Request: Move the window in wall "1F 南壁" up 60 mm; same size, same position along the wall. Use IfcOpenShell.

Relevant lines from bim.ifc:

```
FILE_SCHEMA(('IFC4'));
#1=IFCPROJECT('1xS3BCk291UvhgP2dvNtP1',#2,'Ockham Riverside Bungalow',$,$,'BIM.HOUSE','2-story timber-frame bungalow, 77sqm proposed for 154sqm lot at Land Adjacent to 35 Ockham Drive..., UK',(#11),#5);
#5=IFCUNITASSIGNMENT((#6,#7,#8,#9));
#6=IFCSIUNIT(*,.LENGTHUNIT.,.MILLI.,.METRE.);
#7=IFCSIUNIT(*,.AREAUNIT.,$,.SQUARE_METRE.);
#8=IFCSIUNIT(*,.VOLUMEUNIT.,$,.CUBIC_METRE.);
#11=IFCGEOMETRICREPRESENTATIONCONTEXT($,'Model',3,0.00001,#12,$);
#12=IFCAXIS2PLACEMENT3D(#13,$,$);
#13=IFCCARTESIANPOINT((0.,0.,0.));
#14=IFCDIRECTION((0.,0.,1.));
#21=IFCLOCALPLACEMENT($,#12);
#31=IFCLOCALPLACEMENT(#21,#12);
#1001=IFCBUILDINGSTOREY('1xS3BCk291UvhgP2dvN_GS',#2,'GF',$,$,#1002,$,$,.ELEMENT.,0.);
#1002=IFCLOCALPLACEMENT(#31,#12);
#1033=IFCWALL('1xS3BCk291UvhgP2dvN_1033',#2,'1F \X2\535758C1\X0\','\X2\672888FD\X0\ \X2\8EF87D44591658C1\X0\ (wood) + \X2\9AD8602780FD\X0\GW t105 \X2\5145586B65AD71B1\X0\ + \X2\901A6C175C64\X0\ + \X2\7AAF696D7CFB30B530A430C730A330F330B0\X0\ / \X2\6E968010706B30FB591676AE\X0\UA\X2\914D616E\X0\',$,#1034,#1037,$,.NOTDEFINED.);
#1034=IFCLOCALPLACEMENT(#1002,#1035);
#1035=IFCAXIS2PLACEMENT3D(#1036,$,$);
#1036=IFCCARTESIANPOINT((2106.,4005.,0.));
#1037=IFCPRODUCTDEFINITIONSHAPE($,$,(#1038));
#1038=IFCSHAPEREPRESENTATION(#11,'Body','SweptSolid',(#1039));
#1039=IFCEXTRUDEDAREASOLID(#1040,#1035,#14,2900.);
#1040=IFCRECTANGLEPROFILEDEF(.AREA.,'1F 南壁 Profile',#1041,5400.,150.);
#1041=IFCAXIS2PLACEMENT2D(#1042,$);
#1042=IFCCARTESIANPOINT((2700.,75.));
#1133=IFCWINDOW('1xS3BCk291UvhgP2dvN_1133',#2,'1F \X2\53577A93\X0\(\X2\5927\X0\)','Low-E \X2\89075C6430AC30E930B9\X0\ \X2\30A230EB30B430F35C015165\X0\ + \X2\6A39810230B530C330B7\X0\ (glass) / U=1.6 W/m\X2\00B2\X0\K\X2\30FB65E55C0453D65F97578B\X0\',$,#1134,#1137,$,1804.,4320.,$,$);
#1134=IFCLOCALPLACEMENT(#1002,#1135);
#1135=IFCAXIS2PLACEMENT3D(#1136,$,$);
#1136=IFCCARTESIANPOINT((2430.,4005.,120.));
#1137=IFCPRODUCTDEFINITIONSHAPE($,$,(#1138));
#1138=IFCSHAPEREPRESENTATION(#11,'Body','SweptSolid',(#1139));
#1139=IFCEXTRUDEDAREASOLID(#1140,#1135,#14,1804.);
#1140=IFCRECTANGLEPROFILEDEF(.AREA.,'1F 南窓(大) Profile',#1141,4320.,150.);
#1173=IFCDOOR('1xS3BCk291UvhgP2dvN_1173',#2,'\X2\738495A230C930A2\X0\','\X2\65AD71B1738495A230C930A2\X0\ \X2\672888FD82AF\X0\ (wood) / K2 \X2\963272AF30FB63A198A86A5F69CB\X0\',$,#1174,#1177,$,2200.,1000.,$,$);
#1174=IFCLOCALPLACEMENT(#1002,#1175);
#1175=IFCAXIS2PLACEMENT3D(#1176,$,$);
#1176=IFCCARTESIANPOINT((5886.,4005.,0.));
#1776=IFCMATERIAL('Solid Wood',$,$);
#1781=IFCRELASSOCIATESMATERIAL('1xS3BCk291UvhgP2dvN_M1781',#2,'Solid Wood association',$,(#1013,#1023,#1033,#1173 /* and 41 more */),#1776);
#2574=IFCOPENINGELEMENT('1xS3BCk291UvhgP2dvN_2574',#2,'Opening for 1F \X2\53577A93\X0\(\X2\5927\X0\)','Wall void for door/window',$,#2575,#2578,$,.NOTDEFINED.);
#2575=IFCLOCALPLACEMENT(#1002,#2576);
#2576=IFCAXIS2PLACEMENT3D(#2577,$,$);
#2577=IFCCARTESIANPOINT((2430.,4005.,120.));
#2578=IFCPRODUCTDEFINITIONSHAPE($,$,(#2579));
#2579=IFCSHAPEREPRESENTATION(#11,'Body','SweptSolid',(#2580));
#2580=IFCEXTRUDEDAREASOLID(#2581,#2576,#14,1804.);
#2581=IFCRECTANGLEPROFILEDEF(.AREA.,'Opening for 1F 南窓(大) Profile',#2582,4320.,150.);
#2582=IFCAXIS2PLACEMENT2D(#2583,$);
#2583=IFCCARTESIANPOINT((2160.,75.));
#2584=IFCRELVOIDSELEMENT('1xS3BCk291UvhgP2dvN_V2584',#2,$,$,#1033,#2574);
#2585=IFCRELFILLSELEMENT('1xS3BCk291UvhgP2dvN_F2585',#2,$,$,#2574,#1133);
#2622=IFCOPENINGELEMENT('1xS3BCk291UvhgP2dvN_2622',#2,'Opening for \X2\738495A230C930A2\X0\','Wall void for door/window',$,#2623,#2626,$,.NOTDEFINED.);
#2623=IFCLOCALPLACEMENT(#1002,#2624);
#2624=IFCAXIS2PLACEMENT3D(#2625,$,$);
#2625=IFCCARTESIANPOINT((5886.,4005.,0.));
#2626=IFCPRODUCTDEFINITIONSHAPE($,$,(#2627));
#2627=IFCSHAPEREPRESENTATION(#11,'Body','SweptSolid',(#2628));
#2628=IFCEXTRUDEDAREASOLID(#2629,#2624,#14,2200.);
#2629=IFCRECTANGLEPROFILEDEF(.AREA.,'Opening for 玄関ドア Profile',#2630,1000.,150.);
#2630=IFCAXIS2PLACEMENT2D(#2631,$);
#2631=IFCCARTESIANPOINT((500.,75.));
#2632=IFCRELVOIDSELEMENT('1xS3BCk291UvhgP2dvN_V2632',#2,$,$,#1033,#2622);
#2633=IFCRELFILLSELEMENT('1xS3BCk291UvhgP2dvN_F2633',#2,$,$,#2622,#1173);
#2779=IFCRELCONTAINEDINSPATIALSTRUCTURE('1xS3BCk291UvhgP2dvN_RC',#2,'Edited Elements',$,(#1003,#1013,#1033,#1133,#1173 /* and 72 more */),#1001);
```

```python
import numpy as np
import ifcopenshell
import ifcopenshell.api.geometry
import ifcopenshell.util.placement
import ifcopenshell.util.unit

model = ifcopenshell.open("bim.ifc")
unit_scale = ifcopenshell.util.unit.calculate_unit_scale(model)

window = model.by_guid("1xS3BCk291UvhgP2dvN_1133")
opening = window.FillsVoids[0].RelatingOpeningElement
dz = 0.06 / unit_scale

shift = np.array([0.0, 0.0, dz])
# The window is not placed relative to its opening, so move both.
for product in (opening, window):
    matrix = ifcopenshell.util.placement.get_local_placement(product.ObjectPlacement)
    matrix[:3, 3] += shift
    ifcopenshell.api.geometry.edit_object_placement(model, product=product, matrix=matrix, is_si=False)

print(f"moved by {dz * unit_scale:+.3f} m")

model.write("bim_updated.ifc")
```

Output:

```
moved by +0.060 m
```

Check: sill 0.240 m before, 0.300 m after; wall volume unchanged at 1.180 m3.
